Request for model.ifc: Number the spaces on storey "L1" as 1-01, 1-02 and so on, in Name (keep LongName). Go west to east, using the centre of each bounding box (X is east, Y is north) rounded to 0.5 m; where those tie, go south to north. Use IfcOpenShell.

First a look at what the model holds.

```python
import ifcopenshell
import ifcopenshell.util.element
import ifcopenshell.util.placement

model = ifcopenshell.open("model.ifc")
print(model.schema)
storey = next(s for s in model.by_type("IfcBuildingStorey") if s.Name == "L1")
spaces = [e for e in ifcopenshell.util.element.get_decomposition(storey) if e.is_a("IfcSpace")]
for e in sorted(spaces, key=lambda e: e.id()):
    origin = ifcopenshell.util.placement.get_local_placement(e.ObjectPlacement)[:3, 3]
    print(e.id(), e.Name, e.LongName, origin.round(2) + 0.0, sep=" | ")
```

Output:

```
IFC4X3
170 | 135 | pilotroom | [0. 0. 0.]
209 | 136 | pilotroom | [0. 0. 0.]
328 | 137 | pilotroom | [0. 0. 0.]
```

```python
import ifcopenshell
import ifcopenshell.geom
import ifcopenshell.util.element
import ifcopenshell.util.shape

model = ifcopenshell.open("model.ifc")
settings = ifcopenshell.geom.settings()
settings.set("use-world-coords", True)


def centre(element):
    shape = ifcopenshell.geom.create_shape(settings, element)
    return ifcopenshell.util.shape.get_bbox_centroid(shape.geometry)


storey = next(s for s in model.by_type("IfcBuildingStorey") if s.Name == "L1")
spaces = [e for e in ifcopenshell.util.element.get_decomposition(storey) if e.is_a("IfcSpace")]

# Insertion points can sit at a corner or the storey origin, so sort by the geometry (in metres).
centres = {e: centre(e) for e in spaces}
spaces.sort(key=lambda e: (round(centres[e][0] / 0.5), centres[e][1]))

for i, e in enumerate(spaces, start=1):
    number = f"1-{i:02d}"
    e.Name = number
    print(e.id(), number)

model.write("model-out.ifc")
```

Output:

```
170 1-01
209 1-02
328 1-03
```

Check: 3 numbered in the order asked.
